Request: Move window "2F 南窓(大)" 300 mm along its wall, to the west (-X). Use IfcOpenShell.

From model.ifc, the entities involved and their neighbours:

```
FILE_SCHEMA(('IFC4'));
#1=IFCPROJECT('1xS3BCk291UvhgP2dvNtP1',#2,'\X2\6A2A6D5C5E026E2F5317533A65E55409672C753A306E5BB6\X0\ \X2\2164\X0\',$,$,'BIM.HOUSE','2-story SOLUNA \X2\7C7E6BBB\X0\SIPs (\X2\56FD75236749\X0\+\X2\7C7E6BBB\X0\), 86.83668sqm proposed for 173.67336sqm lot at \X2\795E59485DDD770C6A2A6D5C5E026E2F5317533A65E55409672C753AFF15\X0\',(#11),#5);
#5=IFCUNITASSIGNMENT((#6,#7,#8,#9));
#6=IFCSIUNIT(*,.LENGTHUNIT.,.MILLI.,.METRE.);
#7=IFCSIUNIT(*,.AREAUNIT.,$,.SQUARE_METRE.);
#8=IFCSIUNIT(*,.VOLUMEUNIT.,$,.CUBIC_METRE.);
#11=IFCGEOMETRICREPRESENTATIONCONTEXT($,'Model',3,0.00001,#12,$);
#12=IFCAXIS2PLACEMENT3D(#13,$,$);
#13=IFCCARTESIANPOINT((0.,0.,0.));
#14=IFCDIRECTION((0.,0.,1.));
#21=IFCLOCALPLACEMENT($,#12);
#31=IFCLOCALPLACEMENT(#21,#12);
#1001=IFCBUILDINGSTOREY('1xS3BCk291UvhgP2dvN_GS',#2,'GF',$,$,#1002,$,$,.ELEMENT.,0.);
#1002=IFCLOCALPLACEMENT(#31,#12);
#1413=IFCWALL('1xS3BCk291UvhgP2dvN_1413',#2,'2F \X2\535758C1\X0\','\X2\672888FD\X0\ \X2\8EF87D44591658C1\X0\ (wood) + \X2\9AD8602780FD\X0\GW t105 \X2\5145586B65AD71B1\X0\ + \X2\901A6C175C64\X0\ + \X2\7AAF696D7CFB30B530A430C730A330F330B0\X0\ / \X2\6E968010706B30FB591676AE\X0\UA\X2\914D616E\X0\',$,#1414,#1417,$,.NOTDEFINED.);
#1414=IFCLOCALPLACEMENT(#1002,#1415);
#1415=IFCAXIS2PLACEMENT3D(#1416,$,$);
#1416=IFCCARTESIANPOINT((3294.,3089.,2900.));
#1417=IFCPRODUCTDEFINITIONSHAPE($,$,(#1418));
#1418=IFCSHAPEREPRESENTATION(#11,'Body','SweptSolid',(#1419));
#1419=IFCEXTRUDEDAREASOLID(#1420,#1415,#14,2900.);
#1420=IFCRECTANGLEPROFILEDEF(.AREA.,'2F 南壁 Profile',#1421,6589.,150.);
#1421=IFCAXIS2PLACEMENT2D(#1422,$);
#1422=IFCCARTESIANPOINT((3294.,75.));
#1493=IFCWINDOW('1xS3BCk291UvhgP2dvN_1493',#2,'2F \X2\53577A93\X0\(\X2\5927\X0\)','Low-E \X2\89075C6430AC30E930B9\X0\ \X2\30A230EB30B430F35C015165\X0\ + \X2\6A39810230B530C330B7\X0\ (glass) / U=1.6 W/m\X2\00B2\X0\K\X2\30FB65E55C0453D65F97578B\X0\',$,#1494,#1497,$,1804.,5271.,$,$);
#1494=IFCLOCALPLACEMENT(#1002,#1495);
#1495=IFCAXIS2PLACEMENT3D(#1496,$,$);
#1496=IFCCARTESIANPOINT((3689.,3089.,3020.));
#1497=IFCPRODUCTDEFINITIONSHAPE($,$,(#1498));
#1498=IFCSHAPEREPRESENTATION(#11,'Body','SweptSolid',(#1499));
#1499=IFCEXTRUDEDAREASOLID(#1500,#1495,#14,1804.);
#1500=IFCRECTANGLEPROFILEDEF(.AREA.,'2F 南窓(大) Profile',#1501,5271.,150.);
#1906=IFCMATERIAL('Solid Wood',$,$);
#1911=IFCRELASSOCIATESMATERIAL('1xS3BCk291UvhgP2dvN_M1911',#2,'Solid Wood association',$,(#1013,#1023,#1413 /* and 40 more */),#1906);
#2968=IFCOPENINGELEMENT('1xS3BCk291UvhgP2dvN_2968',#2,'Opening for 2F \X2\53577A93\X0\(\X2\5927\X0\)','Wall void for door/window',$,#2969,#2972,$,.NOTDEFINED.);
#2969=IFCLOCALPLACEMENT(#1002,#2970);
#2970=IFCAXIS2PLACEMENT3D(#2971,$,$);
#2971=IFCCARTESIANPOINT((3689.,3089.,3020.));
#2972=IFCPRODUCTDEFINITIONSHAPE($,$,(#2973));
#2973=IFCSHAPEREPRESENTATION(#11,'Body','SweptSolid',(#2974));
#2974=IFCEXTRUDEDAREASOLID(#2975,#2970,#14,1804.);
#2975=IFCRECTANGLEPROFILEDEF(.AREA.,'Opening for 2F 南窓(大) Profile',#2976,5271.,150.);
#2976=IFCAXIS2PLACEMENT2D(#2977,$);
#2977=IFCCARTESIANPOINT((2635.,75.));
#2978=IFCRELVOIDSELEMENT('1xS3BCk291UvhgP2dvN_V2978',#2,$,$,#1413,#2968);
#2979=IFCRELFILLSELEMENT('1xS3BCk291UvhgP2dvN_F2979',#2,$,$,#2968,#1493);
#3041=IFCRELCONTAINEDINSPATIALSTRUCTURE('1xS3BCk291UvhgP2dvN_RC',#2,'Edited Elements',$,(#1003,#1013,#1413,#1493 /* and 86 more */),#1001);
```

```python
import ifcopenshell
import ifcopenshell.api.geometry
import ifcopenshell.util.placement

model = ifcopenshell.open("model.ifc")

window = model.by_guid("1xS3BCk291UvhgP2dvN_1493")
opening = window.FillsVoids[0].RelatingOpeningElement
wall = opening.VoidsElements[0].RelatingBuildingElement

wall_matrix = ifcopenshell.util.placement.get_local_placement(wall.ObjectPlacement)
shift = wall_matrix[:3, 0] * -300.0
before = ifcopenshell.util.placement.get_local_placement(window.ObjectPlacement)[:3, 3].copy()

# The window is not placed relative to its opening, so move both.
for product in (opening, window):
    matrix = ifcopenshell.util.placement.get_local_placement(product.ObjectPlacement)
    matrix[:3, 3] += shift
    ifcopenshell.api.geometry.edit_object_placement(model, product=product, matrix=matrix, is_si=False)

after = ifcopenshell.util.placement.get_local_placement(window.ObjectPlacement)[:3, 3]
print("window moved by", (after - before).round(3) + 0.0)

model.write("model_rev.ifc")
```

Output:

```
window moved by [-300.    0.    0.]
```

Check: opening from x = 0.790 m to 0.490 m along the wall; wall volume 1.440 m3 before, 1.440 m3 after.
